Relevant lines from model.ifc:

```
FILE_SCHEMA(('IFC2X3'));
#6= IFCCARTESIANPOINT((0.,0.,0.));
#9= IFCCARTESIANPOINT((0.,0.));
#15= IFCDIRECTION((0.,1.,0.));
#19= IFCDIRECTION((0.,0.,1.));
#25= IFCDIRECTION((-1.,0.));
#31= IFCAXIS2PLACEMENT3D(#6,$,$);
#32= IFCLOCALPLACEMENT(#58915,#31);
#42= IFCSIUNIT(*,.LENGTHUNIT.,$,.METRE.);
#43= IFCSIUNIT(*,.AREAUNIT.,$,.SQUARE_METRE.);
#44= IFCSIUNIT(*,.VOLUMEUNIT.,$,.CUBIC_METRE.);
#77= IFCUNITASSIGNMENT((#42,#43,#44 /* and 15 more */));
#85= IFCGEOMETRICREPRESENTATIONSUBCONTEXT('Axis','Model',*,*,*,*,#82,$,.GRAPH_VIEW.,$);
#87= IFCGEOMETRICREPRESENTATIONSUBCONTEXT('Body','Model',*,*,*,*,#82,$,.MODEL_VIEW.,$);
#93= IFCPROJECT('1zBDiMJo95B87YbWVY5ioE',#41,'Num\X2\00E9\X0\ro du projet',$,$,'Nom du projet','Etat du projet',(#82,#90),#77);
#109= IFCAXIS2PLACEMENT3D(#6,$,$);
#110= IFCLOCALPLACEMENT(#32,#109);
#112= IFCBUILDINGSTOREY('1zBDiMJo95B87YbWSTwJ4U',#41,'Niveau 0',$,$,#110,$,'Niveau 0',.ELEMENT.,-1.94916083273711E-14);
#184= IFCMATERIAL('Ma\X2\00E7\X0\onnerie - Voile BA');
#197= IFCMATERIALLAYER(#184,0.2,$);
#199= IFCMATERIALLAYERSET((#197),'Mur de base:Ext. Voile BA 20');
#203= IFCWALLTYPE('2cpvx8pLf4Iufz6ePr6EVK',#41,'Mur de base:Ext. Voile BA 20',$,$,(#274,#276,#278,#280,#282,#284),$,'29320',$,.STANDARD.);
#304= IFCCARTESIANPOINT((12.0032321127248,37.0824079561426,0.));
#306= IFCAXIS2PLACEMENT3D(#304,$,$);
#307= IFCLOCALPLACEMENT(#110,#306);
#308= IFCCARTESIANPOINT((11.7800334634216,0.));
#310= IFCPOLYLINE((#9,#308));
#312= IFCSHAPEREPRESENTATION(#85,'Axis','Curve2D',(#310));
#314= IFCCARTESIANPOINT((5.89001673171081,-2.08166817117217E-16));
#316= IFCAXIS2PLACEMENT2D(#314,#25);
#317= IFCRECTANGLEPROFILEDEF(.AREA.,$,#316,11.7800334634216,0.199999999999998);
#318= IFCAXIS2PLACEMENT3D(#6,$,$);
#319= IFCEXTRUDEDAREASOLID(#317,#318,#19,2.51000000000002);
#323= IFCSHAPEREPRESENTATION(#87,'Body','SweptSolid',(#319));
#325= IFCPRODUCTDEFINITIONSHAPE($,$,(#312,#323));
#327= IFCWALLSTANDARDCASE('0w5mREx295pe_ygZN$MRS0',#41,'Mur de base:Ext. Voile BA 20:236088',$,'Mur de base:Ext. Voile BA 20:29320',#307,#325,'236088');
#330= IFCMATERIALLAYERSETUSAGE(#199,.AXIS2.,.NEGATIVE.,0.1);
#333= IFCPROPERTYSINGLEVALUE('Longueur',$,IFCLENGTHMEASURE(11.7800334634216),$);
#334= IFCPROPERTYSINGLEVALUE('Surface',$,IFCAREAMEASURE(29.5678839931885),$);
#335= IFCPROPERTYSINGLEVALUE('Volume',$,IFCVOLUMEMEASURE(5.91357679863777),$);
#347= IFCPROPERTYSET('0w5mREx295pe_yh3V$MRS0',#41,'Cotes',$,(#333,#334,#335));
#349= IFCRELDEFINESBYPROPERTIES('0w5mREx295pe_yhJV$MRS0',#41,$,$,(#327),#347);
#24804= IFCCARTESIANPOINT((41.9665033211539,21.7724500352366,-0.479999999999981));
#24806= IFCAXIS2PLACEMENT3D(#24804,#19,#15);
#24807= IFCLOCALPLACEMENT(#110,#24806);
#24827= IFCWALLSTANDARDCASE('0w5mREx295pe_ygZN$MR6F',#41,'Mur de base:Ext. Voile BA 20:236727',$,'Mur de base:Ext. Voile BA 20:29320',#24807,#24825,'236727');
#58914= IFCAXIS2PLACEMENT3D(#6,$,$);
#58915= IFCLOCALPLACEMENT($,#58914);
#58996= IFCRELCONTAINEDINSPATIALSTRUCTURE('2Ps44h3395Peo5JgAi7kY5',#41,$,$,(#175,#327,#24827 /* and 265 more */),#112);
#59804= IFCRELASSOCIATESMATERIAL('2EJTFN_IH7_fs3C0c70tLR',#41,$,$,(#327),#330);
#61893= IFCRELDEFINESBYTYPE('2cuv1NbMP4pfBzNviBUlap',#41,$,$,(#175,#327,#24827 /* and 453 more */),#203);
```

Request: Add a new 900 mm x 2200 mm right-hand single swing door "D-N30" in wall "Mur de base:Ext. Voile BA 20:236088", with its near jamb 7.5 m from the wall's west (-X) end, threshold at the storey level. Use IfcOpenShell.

```python
import numpy as np
import ifcopenshell
import ifcopenshell.api.feature
import ifcopenshell.api.geometry
import ifcopenshell.api.pset
import ifcopenshell.api.root
import ifcopenshell.api.spatial
import ifcopenshell.api.type
import ifcopenshell.geom
import ifcopenshell.util.element
import ifcopenshell.util.placement
import ifcopenshell.util.representation
import ifcopenshell.util.shape
import ifcopenshell.util.unit

model = ifcopenshell.open("model.ifc")
unit_scale = ifcopenshell.util.unit.calculate_unit_scale(model)
area_scale = ifcopenshell.util.unit.calculate_unit_scale(model, "AREAUNIT")
volume_scale = ifcopenshell.util.unit.calculate_unit_scale(model, "VOLUMEUNIT")
settings = ifcopenshell.geom.settings()


def volume(element):
    """Net volume in cubic metres, openings subtracted."""
    shape = ifcopenshell.geom.create_shape(settings, element)
    return ifcopenshell.util.shape.get_volume(shape.geometry)


wall = model.by_guid("0w5mREx295pe_ygZN$MRS0")
storey = ifcopenshell.util.element.get_container(wall, ifc_class="IfcBuildingStorey")
context = ifcopenshell.util.representation.get_context(model, "Model", "Body", "MODEL_VIEW")
before = volume(wall)

width, height, from_end, sill = 0.9, 2.2, 7.5, 0.0  # metres

# The wall runs along its own X axis, and the end named is its -X end.
wall_shape = ifcopenshell.geom.create_shape(settings, wall)
x, y, z = ifcopenshell.util.shape.get_vertices(wall_shape.geometry).T
start = x.min() + from_end
face, thickness = float(y.min()), float(y.max() - y.min())
wall_matrix = ifcopenshell.util.placement.get_local_placement(wall.ObjectPlacement)
level = ifcopenshell.util.placement.get_local_placement(storey.ObjectPlacement)[2, 3]


def in_wall(x, y):
    """Placement at x, y metres in the wall's axes, at sill height."""
    matrix = wall_matrix.copy()
    matrix[:, 3] = wall_matrix @ np.array([x / unit_scale, y / unit_scale, 0.0, 1.0])
    matrix[2, 3] = level + sill / unit_scale
    return matrix


# Opening: a box that overshoots both wall faces by 50 mm.
opening = ifcopenshell.api.root.create_entity(model, ifc_class="IfcOpeningElement")
box = ifcopenshell.api.geometry.add_wall_representation(
    model, context=context, length=width, height=height, thickness=thickness + 0.1
)
ifcopenshell.api.geometry.assign_representation(model, product=opening, representation=box)
ifcopenshell.api.geometry.edit_object_placement(model, product=opening, matrix=in_wall(start, face - 0.05), is_si=False)
ifcopenshell.api.feature.add_feature(model, feature=opening, element=wall)

door = ifcopenshell.api.root.create_entity(model, ifc_class="IfcDoor", name="D-N30")
door.OverallWidth, door.OverallHeight = width / unit_scale, height / unit_scale
body = ifcopenshell.api.geometry.add_door_representation(
    model,
    context=context,
    overall_width=door.OverallWidth,
    overall_height=door.OverallHeight,
    operation_type="SINGLE_SWING_RIGHT",
    lining_properties={"LiningDepth": thickness / unit_scale, "ThresholdDepth": thickness / unit_scale},
)
ifcopenshell.api.geometry.assign_representation(model, product=door, representation=body)
ifcopenshell.api.spatial.assign_container(model, products=[door], relating_structure=storey)
fills = ifcopenshell.api.feature.add_filling(model, opening=opening, element=door)
fills.OwnerHistory = door.OwnerHistory  # required in IFC2X3

# IFC2X3 keeps the operation on the door style.
style = ifcopenshell.api.root.create_entity(model, ifc_class="IfcDoorStyle", name="D-N30")
style.OperationType, style.ConstructionType = "SINGLE_SWING_RIGHT", "NOTDEFINED"
style.ParameterTakesPrecedence = style.Sizeable = False
ifcopenshell.api.type.assign_type(model, related_objects=[door], relating_type=style)

# The lining spans the wall, so the door starts at the wall face.
ifcopenshell.api.geometry.edit_object_placement(model, product=door, matrix=in_wall(start, face), is_si=False)

after = volume(wall)

# Update the wall's stored quantities.
pset = model.by_id(ifcopenshell.util.element.get_pset(wall, "Cotes", should_inherit=False)["id"])
ifcopenshell.api.pset.edit_pset(model, pset=pset, properties={
    "Surface": model.create_entity("IfcAreaMeasure", after / thickness / area_scale),
    "Volume": model.create_entity("IfcVolumeMeasure", after / volume_scale),
})

print(f"wall volume {before:.3f} -> {after:.3f} m3")

model.write("model_rev.ifc")
```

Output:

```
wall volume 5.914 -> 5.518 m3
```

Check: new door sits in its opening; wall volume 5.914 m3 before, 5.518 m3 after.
